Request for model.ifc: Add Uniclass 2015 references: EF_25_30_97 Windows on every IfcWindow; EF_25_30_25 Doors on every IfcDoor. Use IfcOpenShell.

First a look at what the model holds.

```python
import ifcopenshell

model = ifcopenshell.open("model.ifc")
print(model.schema)
print("classifications:", [c.Name for c in model.by_type("IfcClassification")])
for ifc_class in ("IfcDoor", "IfcRoof", "IfcStair", "IfcWall", "IfcWindow"):
    print(ifc_class, len(model.by_type(ifc_class)))
```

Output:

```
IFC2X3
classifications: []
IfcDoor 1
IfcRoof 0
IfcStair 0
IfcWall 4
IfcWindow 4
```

```python
import ifcopenshell
import ifcopenshell.api.classification

model = ifcopenshell.open("model.ifc")

# IFC2X3 requires Source and Edition and has no link from the project to the system.
system = model.create_entity("IfcClassification", Source="NBS", Edition="2015", Name="Uniclass 2015")

codes = {
    "IfcWindow": ("EF_25_30_97", "Windows"),
    "IfcDoor": ("EF_25_30_25", "Doors"),
}
for ifc_class, (code, name) in codes.items():
    products = model.by_type(ifc_class)
    ifcopenshell.api.classification.add_reference(
        model, products=products, classification=system, identification=code, name=name
    )
    print(code, len(products))

model.write("model_rev.ifc")
```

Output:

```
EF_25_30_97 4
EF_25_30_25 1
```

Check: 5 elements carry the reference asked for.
